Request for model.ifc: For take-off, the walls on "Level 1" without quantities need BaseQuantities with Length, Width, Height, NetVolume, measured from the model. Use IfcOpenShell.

First a look at what the model holds.

```python
import ifcopenshell
import ifcopenshell.util.element
import ifcopenshell.util.unit

model = ifcopenshell.open("model.ifc")
print(model.schema)
for unit_type in ("LENGTHUNIT", "AREAUNIT", "VOLUMEUNIT"):
    print(unit_type, ifcopenshell.util.unit.calculate_unit_scale(model, unit_type))
storey = next(s for s in model.by_type("IfcBuildingStorey") if s.Name == "Level 1")
walls = [e for e in ifcopenshell.util.element.get_decomposition(storey) if e.is_a("IfcWall")]
for e in sorted(walls, key=lambda e: e.id()):
    print(e.id(), e.is_a(), e.Name, list(ifcopenshell.util.element.get_psets(e, qtos_only=True)), sep=" | ")
```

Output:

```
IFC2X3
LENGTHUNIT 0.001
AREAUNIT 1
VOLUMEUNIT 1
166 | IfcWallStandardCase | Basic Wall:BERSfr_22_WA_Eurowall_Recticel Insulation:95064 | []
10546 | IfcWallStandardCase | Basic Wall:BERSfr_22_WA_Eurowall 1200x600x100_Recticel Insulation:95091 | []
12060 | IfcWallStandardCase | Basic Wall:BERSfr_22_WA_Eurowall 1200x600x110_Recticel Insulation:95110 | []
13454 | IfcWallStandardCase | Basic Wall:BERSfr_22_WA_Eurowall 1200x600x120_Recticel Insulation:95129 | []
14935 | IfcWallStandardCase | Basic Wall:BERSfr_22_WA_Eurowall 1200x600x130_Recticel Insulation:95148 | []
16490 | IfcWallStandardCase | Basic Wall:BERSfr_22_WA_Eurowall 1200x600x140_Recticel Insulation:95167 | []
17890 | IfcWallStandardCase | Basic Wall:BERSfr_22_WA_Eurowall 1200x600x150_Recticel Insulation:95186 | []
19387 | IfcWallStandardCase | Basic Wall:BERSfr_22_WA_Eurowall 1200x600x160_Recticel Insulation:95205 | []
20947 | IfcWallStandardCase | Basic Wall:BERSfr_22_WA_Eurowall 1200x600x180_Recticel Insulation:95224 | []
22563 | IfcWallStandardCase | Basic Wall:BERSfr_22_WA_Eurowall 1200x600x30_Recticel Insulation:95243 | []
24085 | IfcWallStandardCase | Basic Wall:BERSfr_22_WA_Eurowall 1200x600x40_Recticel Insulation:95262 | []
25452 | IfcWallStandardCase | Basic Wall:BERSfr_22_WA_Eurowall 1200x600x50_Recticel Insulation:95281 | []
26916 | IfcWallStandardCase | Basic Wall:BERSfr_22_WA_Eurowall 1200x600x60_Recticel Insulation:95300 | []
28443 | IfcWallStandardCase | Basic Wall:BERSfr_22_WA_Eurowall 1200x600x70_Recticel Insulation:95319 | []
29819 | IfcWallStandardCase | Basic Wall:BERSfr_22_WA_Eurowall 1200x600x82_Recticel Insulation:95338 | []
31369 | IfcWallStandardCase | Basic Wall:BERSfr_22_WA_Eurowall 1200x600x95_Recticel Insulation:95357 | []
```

```python
import ifcopenshell
import ifcopenshell.api.pset
import ifcopenshell.geom
import ifcopenshell.util.element
import ifcopenshell.util.shape
import ifcopenshell.util.unit

model = ifcopenshell.open("model.ifc")
unit_scale = ifcopenshell.util.unit.calculate_unit_scale(model)
volume_scale = ifcopenshell.util.unit.calculate_unit_scale(model, "VOLUMEUNIT")
settings = ifcopenshell.geom.settings()

storey = next(s for s in model.by_type("IfcBuildingStorey") if s.Name == "Level 1")
walls = [e for e in ifcopenshell.util.element.get_decomposition(storey) if e.is_a("IfcWall")]

for e in sorted(walls, key=lambda e: e.id()):
    if ifcopenshell.util.element.get_psets(e, qtos_only=True, should_inherit=False):
        continue
    # Geometry comes back in metres, in the element's own axes.
    shape = ifcopenshell.geom.create_shape(settings, e)
    values = {
        "Length": ifcopenshell.util.shape.get_x(shape.geometry) / unit_scale,
        "Width": ifcopenshell.util.shape.get_y(shape.geometry) / unit_scale,
        "Height": ifcopenshell.util.shape.get_z(shape.geometry) / unit_scale,
        "NetVolume": ifcopenshell.util.shape.get_volume(shape.geometry) / volume_scale,
    }
    qto = ifcopenshell.api.pset.add_qto(model, product=e, name="BaseQuantities")
    ifcopenshell.api.pset.edit_qto(model, qto=qto, properties=values)
    print(e.id(), {k: round(v, 3) for k, v in values.items()})

model.write("model_v2.ifc")
```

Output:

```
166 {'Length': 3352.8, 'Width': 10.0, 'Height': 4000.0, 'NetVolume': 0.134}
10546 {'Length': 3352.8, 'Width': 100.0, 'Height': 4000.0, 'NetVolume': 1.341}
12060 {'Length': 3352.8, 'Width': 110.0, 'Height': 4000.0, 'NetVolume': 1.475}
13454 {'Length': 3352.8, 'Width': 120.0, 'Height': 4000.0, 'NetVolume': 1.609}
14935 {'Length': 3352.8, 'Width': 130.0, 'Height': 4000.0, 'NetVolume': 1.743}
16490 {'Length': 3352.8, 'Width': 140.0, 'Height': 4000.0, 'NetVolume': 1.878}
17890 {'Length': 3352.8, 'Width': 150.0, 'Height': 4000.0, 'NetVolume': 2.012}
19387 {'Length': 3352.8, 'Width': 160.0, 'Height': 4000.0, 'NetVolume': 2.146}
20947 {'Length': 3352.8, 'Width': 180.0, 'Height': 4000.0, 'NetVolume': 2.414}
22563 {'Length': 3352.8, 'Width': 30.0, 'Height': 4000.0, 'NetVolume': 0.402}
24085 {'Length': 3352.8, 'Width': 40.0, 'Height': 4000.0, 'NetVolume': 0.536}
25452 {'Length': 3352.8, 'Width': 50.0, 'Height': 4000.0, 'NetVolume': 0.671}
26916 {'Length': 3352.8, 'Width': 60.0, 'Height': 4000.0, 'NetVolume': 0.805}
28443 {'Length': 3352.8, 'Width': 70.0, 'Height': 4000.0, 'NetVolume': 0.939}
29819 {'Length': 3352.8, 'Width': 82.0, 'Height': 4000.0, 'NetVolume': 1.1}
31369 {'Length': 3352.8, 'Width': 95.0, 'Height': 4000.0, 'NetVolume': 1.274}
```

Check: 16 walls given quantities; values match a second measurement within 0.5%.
